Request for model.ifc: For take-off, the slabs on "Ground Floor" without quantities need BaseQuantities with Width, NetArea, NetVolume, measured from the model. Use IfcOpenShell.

First a look at what the model holds.

```python
import ifcopenshell
import ifcopenshell.util.element
import ifcopenshell.util.unit

model = ifcopenshell.open("model.ifc")
print(model.schema)
for unit_type in ("LENGTHUNIT", "AREAUNIT", "VOLUMEUNIT"):
    print(unit_type, ifcopenshell.util.unit.calculate_unit_scale(model, unit_type))
storey = next(s for s in model.by_type("IfcBuildingStorey") if s.Name == "Ground Floor")
slabs = [e for e in ifcopenshell.util.element.get_decomposition(storey) if e.is_a("IfcSlab")]
for e in sorted(slabs, key=lambda e: e.id()):
    print(e.id(), e.is_a(), e.Name, list(ifcopenshell.util.element.get_psets(e, qtos_only=True)), sep=" | ")
```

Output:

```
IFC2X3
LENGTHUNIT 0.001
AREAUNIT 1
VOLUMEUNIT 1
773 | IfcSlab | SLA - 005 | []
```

```python
import ifcopenshell
import ifcopenshell.api.pset
import ifcopenshell.geom
import ifcopenshell.util.element
import ifcopenshell.util.shape
import ifcopenshell.util.unit

model = ifcopenshell.open("model.ifc")
unit_scale = ifcopenshell.util.unit.calculate_unit_scale(model)
area_scale = ifcopenshell.util.unit.calculate_unit_scale(model, "AREAUNIT")
volume_scale = ifcopenshell.util.unit.calculate_unit_scale(model, "VOLUMEUNIT")
settings = ifcopenshell.geom.settings()

storey = next(s for s in model.by_type("IfcBuildingStorey") if s.Name == "Ground Floor")
slabs = [e for e in ifcopenshell.util.element.get_decomposition(storey) if e.is_a("IfcSlab")]

for e in sorted(slabs, key=lambda e: e.id()):
    if ifcopenshell.util.element.get_psets(e, qtos_only=True, should_inherit=False):
        continue
    # Geometry comes back in metres, in the element's own axes.
    shape = ifcopenshell.geom.create_shape(settings, e)
    values = {
        "Width": ifcopenshell.util.shape.get_z(shape.geometry) / unit_scale,
        "NetArea": ifcopenshell.util.shape.get_footprint_area(shape.geometry) / area_scale,
        "NetVolume": ifcopenshell.util.shape.get_volume(shape.geometry) / volume_scale,
    }
    qto = ifcopenshell.api.pset.add_qto(model, product=e, name="BaseQuantities")
    ifcopenshell.api.pset.edit_qto(model, qto=qto, properties=values)
    print(e.id(), {k: round(v, 3) for k, v in values.items()})

model.write("model_edited.ifc")
```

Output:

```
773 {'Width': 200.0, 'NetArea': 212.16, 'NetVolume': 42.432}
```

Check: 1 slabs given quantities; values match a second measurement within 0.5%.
